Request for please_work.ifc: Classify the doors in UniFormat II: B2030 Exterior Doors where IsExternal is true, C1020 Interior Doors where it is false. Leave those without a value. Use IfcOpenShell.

First a look at what the model holds.

```python
import ifcopenshell
import ifcopenshell.util.element

model = ifcopenshell.open("please_work.ifc")
print(model.schema)
print("classifications:", [c.Name for c in model.by_type("IfcClassification")])
values = [ifcopenshell.util.element.get_pset(e, "Pset_DoorCommon", "IsExternal") for e in model.by_type("IfcDoor")]
for value in (True, False, None):
    print("IsExternal", value, values.count(value))
```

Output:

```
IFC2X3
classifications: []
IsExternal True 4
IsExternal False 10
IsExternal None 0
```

```python
import ifcopenshell
import ifcopenshell.api.classification
import ifcopenshell.util.element

model = ifcopenshell.open("please_work.ifc")

# IFC2X3 requires Source and Edition and has no link from the project to the system.
system = model.create_entity("IfcClassification", Source="ASTM", Edition="E1557", Name="UniFormat II")

doors = model.by_type("IfcDoor")
external = {e: ifcopenshell.util.element.get_pset(e, "Pset_DoorCommon", "IsExternal") for e in doors}
for flag, code, name in ((True, "B2030", "Exterior Doors"), (False, "C1020", "Interior Doors")):
    products = [e for e in doors if external[e] is flag]
    ifcopenshell.api.classification.add_reference(
        model, products=products, classification=system, identification=code, name=name
    )
    print(code, len(products))

model.write("please_work_rev.ifc")
```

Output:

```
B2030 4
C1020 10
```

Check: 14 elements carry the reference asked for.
